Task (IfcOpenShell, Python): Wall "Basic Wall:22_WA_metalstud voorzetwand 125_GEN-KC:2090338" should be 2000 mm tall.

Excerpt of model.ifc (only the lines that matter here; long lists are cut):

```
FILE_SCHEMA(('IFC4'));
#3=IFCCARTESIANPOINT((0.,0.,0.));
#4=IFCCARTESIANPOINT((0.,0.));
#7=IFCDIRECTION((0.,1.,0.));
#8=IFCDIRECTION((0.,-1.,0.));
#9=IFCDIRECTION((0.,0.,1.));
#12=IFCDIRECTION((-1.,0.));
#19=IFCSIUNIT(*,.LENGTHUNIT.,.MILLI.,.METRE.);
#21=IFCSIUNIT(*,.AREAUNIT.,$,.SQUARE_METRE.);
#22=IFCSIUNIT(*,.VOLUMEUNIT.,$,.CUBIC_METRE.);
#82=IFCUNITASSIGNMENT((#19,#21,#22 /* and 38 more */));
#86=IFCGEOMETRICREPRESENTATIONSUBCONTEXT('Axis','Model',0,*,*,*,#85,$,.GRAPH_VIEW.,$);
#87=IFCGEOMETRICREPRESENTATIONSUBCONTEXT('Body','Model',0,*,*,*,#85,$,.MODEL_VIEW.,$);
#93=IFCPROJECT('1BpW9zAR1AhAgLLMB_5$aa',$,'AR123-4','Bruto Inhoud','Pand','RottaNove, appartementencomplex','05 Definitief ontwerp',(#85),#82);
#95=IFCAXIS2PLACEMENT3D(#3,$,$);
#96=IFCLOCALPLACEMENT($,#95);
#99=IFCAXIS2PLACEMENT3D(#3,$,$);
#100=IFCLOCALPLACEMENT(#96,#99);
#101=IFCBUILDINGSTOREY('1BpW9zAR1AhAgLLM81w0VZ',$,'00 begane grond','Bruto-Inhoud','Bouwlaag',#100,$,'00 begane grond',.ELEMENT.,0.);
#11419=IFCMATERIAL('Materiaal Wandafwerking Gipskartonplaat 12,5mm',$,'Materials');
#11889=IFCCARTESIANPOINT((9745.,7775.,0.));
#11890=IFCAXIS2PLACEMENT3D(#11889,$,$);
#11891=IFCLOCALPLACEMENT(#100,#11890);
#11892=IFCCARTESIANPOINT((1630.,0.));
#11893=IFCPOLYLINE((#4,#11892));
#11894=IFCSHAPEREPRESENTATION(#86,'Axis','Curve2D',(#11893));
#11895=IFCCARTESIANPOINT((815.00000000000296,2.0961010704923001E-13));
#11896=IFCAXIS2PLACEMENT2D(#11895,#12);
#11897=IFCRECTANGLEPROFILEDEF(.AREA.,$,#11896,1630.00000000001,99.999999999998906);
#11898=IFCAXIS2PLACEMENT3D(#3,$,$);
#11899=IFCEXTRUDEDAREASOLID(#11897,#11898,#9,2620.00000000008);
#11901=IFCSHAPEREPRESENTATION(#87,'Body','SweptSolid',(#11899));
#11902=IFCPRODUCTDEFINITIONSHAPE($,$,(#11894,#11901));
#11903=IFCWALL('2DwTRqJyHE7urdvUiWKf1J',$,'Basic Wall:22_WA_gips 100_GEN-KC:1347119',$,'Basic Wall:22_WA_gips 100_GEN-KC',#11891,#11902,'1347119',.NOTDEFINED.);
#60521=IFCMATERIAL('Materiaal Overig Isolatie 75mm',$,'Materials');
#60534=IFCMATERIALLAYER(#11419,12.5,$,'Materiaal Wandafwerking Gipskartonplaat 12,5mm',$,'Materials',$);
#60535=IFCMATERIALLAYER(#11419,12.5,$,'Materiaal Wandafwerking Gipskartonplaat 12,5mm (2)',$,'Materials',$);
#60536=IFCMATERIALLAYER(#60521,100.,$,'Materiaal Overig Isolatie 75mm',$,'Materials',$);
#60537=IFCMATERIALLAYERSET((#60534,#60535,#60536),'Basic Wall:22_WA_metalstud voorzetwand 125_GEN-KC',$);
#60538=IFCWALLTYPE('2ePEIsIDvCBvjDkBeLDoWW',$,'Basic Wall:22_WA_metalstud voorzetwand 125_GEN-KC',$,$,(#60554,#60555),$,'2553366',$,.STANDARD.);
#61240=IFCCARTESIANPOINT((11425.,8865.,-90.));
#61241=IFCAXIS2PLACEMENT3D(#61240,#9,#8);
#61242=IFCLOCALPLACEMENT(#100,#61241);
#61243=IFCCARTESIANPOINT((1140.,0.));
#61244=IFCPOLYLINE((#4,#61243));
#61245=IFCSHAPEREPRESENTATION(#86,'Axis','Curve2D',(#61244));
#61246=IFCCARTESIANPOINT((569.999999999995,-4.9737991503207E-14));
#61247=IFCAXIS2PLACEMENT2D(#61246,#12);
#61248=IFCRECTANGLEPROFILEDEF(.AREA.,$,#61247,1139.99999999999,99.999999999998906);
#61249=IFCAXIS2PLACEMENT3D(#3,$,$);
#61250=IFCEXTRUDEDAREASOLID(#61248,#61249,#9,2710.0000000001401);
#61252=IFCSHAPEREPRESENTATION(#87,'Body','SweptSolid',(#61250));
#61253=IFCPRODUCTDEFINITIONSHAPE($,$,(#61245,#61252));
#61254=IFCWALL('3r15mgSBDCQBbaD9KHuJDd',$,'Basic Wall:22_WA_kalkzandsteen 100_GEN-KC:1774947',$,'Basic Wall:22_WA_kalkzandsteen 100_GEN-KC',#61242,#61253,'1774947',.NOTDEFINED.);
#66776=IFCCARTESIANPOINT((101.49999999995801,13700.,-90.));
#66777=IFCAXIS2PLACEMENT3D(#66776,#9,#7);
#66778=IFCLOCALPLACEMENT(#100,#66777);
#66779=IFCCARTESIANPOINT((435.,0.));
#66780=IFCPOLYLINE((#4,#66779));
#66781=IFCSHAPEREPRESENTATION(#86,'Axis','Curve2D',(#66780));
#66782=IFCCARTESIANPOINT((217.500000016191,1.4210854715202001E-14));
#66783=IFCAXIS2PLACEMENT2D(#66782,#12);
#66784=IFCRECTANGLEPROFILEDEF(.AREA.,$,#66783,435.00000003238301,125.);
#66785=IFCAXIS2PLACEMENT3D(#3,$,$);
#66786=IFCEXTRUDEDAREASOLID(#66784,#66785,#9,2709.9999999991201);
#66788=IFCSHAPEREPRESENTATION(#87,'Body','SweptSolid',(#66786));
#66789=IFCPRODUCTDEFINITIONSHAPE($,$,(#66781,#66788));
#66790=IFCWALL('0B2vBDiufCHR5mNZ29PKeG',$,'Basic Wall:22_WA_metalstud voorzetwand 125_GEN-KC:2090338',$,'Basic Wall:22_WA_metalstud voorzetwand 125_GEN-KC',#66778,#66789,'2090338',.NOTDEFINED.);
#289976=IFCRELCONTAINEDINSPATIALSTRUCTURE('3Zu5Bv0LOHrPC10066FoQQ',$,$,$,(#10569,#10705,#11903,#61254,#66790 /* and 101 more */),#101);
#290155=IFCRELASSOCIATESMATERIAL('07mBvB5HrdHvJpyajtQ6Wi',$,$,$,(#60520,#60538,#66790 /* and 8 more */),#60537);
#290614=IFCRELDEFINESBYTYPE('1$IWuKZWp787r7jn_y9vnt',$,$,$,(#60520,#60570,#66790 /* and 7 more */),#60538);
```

```python
import ifcopenshell
import ifcopenshell.geom
import ifcopenshell.util.representation
import ifcopenshell.util.shape

model = ifcopenshell.open("model.ifc")
settings = ifcopenshell.geom.settings()


def volume(element):
    """Net volume in cubic metres, openings subtracted."""
    shape = ifcopenshell.geom.create_shape(settings, element)
    return ifcopenshell.util.shape.get_volume(shape.geometry)


wall = model.by_id(66790)
before = volume(wall)

body = ifcopenshell.util.representation.get_representation(wall, "Model", "Body")
solid = body.Items[0]
old_height = solid.Depth
solid.Depth = 2000.0
after = volume(wall)

print(f"height {old_height:g} -> {solid.Depth:g}, volume {before:.3f} -> {after:.3f} m3")

model.write("model_updated.ifc")
```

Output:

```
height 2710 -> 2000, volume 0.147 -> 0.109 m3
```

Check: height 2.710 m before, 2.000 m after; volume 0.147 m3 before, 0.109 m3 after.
